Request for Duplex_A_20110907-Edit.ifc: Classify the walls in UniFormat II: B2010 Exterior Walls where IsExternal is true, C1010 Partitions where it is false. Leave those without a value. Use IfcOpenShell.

First a look at what the model holds.

```python
import ifcopenshell
import ifcopenshell.util.element

model = ifcopenshell.open("Duplex_A_20110907-Edit.ifc")
print(model.schema)
print("classifications:", [c.Name for c in model.by_type("IfcClassification")])
values = [ifcopenshell.util.element.get_pset(e, "Pset_WallCommon", "IsExternal") for e in model.by_type("IfcWall")]
for value in (True, False, None):
    print("IsExternal", value, values.count(value))
```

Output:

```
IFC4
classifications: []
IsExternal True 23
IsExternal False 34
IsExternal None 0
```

```python
import ifcopenshell
import ifcopenshell.api.classification
import ifcopenshell.util.element

model = ifcopenshell.open("Duplex_A_20110907-Edit.ifc")

system = ifcopenshell.api.classification.add_classification(model, classification="UniFormat II")

walls = model.by_type("IfcWall")
external = {e: ifcopenshell.util.element.get_pset(e, "Pset_WallCommon", "IsExternal") for e in walls}
for flag, code, name in ((True, "B2010", "Exterior Walls"), (False, "C1010", "Partitions")):
    products = [e for e in walls if external[e] is flag]
    ifcopenshell.api.classification.add_reference(
        model, products=products, classification=system, identification=code, name=name
    )
    print(code, len(products))

model.write("Duplex_A_20110907-Edit_updated.ifc")
```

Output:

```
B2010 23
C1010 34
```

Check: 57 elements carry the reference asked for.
